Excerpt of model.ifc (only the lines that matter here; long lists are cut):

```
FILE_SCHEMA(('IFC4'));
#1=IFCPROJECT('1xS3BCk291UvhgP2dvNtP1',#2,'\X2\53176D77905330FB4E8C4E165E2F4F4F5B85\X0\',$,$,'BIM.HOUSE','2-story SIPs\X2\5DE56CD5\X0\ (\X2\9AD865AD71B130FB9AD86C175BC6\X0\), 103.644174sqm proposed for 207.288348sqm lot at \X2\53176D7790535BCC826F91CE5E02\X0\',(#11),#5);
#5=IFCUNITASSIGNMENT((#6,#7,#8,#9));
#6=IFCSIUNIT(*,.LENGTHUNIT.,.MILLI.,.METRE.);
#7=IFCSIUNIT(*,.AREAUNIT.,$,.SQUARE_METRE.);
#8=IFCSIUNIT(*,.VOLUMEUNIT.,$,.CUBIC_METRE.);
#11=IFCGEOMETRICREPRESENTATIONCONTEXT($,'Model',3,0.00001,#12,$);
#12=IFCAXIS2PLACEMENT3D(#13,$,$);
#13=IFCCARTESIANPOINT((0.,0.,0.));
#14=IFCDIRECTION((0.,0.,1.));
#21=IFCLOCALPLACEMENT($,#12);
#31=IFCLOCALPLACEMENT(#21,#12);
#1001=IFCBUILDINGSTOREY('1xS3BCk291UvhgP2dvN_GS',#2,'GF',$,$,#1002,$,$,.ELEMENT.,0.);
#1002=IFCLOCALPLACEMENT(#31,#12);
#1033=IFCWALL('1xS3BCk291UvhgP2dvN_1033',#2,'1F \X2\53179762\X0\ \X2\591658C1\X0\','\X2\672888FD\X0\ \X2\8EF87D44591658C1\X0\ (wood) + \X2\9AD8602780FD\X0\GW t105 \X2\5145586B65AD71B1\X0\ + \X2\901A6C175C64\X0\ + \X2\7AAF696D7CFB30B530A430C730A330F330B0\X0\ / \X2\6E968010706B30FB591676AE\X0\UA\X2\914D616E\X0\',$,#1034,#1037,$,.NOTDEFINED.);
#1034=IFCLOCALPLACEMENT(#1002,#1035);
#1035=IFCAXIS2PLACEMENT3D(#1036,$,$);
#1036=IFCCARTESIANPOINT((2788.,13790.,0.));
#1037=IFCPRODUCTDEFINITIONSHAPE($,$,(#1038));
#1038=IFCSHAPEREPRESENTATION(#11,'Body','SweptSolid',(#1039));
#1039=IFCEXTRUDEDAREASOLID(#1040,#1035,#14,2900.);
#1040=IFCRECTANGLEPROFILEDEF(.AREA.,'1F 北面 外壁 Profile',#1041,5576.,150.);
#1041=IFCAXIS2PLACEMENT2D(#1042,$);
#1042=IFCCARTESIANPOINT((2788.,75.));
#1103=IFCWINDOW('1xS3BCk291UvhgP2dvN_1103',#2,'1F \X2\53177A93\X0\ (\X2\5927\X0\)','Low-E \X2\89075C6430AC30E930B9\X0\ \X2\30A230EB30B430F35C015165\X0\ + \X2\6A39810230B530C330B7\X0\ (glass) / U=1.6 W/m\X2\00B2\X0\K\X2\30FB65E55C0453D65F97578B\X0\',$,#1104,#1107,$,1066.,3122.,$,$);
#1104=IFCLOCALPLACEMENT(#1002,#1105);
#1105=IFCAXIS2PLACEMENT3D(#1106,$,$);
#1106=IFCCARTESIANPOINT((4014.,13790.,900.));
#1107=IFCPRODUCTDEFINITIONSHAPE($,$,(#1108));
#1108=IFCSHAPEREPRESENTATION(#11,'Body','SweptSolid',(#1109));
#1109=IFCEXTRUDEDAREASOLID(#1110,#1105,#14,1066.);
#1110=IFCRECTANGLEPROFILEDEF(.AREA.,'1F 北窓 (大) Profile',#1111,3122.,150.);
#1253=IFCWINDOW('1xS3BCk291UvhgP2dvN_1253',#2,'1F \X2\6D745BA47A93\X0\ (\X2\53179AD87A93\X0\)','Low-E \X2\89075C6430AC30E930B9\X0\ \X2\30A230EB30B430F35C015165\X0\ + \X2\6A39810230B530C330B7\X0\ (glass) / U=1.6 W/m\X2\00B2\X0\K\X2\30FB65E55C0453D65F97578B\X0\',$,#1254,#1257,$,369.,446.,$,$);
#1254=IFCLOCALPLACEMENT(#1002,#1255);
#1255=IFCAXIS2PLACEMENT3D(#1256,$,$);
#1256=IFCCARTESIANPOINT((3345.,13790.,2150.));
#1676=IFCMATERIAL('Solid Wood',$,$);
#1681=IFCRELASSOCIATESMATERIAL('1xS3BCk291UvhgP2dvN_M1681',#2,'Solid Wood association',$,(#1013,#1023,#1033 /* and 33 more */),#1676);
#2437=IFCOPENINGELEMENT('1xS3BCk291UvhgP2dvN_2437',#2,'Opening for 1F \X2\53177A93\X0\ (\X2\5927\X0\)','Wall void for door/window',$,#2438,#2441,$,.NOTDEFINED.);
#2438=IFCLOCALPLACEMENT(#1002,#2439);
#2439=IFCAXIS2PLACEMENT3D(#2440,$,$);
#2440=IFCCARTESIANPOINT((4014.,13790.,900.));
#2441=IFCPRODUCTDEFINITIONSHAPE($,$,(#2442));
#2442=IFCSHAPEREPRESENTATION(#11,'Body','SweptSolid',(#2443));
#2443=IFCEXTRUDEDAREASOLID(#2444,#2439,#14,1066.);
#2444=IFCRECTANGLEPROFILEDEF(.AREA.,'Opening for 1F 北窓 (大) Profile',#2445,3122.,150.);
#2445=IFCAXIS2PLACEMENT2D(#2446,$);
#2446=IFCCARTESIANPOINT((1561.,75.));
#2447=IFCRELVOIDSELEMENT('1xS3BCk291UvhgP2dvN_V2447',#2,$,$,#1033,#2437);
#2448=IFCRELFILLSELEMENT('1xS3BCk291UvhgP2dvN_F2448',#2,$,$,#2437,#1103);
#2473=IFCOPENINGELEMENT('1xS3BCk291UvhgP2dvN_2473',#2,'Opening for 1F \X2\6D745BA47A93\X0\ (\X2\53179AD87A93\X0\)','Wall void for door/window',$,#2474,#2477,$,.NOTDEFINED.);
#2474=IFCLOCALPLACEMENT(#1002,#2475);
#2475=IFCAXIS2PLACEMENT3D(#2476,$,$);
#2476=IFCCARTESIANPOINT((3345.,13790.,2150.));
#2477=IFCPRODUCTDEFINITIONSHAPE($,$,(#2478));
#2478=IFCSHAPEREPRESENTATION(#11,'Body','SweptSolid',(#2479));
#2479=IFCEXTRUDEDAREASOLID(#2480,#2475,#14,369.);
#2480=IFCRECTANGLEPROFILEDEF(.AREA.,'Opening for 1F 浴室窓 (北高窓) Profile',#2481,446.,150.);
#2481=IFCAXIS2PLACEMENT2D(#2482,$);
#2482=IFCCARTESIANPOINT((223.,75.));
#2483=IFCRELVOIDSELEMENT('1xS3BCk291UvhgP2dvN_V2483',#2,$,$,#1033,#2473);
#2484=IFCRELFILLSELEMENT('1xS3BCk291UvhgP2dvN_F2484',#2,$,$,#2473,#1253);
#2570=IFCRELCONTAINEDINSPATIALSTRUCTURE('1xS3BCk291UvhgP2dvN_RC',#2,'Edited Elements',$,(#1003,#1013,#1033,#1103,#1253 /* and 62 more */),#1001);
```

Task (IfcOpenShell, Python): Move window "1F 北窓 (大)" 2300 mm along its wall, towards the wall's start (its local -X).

```python
import ifcopenshell
import ifcopenshell.api.geometry
import ifcopenshell.util.placement

model = ifcopenshell.open("model.ifc")

window = model.by_id(1103)
opening = window.FillsVoids[0].RelatingOpeningElement
wall = opening.VoidsElements[0].RelatingBuildingElement

wall_matrix = ifcopenshell.util.placement.get_local_placement(wall.ObjectPlacement)
shift = wall_matrix[:3, 0] * -2300.0
before = ifcopenshell.util.placement.get_local_placement(window.ObjectPlacement)[:3, 3].copy()

# The window is not placed relative to its opening, so move both.
for product in (opening, window):
    matrix = ifcopenshell.util.placement.get_local_placement(product.ObjectPlacement)
    matrix[:3, 3] += shift
    ifcopenshell.api.geometry.edit_object_placement(model, product=product, matrix=matrix, is_si=False)

after = ifcopenshell.util.placement.get_local_placement(window.ObjectPlacement)[:3, 3]
print("window moved by", (after - before).round(3) + 0.0)

model.write("model_v2.ifc")
```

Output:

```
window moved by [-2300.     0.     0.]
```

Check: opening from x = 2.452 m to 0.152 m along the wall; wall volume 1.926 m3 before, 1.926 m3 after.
